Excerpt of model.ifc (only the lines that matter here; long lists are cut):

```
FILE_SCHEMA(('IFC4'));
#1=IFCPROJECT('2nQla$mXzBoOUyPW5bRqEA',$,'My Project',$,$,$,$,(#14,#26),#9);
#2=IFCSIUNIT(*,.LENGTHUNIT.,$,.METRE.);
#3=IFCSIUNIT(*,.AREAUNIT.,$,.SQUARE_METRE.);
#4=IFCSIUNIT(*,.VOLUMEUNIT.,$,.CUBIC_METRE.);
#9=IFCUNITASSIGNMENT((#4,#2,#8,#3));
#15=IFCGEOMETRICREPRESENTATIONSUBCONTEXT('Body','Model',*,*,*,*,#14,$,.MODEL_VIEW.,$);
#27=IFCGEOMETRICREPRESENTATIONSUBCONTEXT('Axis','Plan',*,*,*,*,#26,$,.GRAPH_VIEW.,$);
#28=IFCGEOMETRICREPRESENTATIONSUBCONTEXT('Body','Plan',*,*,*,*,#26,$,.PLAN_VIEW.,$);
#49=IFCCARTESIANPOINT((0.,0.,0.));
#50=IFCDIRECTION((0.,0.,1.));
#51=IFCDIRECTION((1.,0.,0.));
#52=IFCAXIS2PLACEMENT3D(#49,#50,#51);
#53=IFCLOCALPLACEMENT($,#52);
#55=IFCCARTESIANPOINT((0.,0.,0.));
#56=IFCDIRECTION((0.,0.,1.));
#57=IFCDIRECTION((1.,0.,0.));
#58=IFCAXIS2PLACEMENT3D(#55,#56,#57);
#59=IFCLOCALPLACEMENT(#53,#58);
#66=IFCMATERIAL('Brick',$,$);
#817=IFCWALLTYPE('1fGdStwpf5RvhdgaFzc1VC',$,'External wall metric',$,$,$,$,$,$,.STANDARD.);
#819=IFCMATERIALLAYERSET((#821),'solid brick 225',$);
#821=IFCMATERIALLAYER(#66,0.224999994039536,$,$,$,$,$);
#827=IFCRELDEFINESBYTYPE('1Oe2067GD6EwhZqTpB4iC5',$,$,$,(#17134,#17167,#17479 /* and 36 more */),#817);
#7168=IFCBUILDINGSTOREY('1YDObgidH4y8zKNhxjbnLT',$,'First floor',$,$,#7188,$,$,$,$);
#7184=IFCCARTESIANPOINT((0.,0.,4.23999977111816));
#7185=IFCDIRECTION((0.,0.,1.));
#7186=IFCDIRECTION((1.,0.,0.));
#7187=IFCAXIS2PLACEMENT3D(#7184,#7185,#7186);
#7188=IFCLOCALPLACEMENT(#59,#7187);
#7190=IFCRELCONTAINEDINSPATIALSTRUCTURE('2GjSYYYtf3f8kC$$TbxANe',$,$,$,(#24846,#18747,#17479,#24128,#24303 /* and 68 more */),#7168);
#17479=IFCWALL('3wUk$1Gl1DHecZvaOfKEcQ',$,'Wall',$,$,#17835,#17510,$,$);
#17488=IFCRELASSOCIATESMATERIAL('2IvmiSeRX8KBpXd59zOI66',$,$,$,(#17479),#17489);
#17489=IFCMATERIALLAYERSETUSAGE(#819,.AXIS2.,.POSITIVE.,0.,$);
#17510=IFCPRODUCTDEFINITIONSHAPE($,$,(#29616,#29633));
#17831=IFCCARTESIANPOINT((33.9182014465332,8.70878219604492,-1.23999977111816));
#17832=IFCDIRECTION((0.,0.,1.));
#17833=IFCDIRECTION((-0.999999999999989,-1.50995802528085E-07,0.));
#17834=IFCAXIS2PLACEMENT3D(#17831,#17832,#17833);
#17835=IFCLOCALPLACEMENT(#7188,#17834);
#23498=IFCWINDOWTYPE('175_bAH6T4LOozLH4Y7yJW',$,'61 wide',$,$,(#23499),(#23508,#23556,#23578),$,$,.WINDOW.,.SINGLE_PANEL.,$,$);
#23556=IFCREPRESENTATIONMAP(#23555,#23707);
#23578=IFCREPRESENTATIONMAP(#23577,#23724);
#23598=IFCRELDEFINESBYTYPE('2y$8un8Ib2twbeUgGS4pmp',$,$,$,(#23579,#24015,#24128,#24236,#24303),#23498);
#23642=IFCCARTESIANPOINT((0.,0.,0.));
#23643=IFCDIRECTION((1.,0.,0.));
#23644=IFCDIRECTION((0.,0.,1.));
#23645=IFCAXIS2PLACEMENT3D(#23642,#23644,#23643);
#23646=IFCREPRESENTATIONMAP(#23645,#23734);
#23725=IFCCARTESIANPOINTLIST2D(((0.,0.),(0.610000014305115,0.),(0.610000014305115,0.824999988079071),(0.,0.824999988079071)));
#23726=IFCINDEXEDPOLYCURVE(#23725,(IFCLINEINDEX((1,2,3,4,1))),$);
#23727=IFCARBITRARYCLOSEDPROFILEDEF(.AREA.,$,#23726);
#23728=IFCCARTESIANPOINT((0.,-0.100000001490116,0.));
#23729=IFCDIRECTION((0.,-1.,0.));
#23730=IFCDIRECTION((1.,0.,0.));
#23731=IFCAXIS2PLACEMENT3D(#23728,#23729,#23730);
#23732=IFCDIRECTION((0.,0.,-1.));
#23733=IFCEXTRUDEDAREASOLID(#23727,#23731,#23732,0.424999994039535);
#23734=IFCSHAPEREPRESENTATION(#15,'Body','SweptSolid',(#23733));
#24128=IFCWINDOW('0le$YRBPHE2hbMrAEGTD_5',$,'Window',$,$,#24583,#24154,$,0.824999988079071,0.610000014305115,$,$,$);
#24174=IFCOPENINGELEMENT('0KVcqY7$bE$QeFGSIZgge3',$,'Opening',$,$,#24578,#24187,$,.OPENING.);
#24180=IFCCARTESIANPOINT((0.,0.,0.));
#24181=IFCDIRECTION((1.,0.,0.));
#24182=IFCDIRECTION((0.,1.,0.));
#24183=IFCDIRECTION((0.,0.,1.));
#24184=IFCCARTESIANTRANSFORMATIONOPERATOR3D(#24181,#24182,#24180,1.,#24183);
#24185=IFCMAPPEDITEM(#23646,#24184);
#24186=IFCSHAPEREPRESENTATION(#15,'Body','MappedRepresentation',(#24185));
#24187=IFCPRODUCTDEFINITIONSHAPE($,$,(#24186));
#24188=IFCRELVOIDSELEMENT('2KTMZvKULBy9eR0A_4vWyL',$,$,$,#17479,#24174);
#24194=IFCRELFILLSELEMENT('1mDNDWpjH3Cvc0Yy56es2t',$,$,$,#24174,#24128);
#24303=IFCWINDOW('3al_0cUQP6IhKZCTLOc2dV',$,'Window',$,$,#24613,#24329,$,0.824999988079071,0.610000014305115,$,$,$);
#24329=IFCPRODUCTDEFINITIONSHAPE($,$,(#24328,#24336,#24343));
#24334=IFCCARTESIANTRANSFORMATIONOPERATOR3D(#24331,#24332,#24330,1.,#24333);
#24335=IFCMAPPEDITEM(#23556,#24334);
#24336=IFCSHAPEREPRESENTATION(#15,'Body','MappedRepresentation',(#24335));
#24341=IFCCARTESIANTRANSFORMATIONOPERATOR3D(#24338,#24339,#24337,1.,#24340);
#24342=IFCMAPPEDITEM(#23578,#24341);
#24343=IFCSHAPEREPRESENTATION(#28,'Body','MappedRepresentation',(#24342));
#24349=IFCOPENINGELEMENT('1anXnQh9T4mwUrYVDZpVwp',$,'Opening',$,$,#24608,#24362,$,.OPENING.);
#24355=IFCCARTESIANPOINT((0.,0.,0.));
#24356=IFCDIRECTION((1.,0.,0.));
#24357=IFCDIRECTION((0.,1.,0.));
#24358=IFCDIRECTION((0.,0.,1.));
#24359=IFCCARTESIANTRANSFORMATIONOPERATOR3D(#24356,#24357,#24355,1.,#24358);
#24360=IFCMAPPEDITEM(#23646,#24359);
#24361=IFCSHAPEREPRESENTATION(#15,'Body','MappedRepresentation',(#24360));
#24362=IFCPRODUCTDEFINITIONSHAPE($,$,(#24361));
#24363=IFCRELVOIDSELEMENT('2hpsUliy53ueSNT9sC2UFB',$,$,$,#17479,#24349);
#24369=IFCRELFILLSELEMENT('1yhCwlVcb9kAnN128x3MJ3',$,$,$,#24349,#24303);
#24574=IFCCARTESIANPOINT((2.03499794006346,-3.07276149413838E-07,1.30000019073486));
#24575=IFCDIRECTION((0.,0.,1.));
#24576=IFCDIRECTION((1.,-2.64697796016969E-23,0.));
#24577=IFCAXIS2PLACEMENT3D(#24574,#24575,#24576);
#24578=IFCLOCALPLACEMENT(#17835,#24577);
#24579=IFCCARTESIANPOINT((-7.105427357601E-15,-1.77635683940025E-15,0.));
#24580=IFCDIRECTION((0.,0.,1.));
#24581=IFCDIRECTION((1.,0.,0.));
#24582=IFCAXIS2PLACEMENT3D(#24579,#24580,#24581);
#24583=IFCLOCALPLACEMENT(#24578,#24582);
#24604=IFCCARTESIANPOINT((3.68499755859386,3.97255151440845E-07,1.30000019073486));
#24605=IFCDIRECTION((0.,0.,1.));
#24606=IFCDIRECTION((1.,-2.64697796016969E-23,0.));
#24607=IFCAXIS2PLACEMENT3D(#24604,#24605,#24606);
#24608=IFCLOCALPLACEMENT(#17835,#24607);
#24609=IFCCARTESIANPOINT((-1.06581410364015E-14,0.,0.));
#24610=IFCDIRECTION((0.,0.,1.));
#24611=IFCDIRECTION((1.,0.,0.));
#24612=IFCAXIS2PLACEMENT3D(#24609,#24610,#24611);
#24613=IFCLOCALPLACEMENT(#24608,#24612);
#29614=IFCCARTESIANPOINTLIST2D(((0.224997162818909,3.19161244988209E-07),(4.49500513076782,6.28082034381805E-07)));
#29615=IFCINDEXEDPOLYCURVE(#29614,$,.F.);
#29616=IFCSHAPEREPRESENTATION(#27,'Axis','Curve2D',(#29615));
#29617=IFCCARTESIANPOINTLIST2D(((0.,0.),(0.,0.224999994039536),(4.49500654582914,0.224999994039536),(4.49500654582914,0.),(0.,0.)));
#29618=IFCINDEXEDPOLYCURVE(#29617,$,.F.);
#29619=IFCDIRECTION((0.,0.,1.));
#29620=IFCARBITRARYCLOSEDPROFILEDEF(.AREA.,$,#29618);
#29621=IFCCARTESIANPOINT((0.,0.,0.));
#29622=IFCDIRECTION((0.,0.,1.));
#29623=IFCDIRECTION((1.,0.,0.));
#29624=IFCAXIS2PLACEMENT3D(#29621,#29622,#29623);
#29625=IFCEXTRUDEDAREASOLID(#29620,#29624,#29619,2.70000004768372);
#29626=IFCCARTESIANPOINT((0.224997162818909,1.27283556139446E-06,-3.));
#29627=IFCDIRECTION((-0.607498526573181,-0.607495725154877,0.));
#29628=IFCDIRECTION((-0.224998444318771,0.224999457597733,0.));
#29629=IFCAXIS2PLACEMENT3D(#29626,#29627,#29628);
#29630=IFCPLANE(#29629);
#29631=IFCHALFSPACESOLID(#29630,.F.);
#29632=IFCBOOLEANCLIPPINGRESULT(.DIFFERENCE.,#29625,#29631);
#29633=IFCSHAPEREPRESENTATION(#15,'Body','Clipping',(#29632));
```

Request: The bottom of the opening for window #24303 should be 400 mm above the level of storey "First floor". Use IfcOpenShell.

```python
import numpy as np
import ifcopenshell
import ifcopenshell.api.geometry
import ifcopenshell.geom
import ifcopenshell.util.element
import ifcopenshell.util.placement
import ifcopenshell.util.shape
import ifcopenshell.util.unit

model = ifcopenshell.open("model.ifc")
unit_scale = ifcopenshell.util.unit.calculate_unit_scale(model)

window = model.by_guid("3al_0cUQP6IhKZCTLOc2dV")
opening = window.FillsVoids[0].RelatingOpeningElement
storey = ifcopenshell.util.element.get_container(window, ifc_class="IfcBuildingStorey")
level = ifcopenshell.util.placement.get_local_placement(storey.ObjectPlacement)[2, 3]

# The opening's origin need not be at the sill, so measure its lowest point.
shape = ifcopenshell.geom.create_shape(ifcopenshell.geom.settings(), opening)
bottom = ifcopenshell.util.shape.get_shape_bottom_elevation(shape, shape.geometry) / unit_scale
dz = level + 0.4 / unit_scale - bottom

shift = np.array([0.0, 0.0, dz])
# The window is placed relative to its opening, so it follows when the opening moves.
matrix = ifcopenshell.util.placement.get_local_placement(opening.ObjectPlacement)
matrix[:3, 3] += shift
ifcopenshell.api.geometry.edit_object_placement(
    model, product=opening, matrix=matrix, is_si=False, should_transform_children=True
)

print(f"moved by {dz * unit_scale:+.3f} m")

model.write("model_updated.ifc")
```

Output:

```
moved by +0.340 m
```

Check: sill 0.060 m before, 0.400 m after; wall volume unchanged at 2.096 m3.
